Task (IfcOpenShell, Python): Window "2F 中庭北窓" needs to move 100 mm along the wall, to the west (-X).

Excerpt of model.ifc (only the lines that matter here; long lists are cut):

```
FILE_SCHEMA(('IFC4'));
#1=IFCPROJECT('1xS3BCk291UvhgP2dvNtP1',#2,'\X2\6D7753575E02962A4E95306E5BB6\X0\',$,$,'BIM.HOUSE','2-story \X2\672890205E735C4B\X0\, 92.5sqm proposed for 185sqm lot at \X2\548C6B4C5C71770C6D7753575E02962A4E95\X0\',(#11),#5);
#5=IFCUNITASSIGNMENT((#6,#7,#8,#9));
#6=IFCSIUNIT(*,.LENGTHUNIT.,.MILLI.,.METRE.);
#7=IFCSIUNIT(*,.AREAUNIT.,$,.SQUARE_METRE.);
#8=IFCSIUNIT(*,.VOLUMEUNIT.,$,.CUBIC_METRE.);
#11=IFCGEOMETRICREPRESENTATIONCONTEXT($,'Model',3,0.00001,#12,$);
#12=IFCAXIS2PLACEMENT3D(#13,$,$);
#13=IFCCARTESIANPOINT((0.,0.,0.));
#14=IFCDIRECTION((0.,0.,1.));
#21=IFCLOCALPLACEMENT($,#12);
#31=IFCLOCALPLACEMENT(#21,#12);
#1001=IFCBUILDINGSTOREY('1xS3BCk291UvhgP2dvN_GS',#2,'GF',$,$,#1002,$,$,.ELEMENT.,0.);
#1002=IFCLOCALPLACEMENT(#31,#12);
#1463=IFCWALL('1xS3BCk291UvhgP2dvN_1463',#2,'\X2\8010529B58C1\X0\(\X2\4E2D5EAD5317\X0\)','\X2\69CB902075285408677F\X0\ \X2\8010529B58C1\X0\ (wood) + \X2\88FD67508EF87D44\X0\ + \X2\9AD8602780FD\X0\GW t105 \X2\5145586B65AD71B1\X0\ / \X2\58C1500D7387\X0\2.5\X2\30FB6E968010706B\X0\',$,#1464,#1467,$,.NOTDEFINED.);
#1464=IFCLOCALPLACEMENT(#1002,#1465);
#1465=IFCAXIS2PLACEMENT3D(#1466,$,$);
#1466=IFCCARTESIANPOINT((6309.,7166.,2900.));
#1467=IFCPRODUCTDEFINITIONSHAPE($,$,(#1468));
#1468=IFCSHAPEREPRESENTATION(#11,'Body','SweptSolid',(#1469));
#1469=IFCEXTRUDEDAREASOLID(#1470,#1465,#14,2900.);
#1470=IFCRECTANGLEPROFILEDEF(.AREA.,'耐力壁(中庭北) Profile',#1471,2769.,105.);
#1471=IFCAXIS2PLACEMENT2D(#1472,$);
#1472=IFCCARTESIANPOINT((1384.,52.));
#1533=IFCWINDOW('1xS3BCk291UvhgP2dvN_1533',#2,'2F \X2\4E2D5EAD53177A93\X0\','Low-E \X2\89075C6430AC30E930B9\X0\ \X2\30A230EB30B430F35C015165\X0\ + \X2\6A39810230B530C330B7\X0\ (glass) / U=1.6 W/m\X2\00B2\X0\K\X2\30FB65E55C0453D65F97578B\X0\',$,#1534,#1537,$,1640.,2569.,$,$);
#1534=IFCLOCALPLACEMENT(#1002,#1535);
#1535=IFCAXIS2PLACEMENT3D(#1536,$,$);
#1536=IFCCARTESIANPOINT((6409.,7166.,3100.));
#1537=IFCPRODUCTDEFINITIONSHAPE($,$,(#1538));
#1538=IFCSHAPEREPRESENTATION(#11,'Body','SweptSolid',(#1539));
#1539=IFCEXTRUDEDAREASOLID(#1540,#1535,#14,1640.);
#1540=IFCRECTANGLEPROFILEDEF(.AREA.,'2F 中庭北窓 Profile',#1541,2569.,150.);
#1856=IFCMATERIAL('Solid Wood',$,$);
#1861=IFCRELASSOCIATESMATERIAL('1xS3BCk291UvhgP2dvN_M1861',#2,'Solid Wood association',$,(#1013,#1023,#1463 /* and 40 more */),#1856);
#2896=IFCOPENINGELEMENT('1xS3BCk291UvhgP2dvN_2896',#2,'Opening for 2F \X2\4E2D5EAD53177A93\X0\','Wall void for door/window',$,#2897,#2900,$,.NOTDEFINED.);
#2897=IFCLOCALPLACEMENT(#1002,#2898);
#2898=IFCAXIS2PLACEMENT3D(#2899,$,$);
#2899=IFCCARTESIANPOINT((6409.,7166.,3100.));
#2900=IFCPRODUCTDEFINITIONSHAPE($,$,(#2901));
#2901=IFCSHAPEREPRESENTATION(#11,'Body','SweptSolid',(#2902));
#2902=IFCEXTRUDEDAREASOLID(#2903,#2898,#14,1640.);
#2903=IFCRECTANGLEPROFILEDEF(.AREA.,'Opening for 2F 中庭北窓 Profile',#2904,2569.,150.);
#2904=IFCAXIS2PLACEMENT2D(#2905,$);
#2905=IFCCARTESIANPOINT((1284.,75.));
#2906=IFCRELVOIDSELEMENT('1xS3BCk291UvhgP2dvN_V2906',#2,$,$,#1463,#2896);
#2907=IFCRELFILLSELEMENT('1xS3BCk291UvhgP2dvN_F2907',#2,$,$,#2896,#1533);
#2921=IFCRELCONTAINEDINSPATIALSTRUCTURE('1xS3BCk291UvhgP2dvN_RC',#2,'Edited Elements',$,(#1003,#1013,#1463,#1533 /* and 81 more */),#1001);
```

```python
import ifcopenshell
import ifcopenshell.api.geometry
import ifcopenshell.util.placement
import ifcopenshell.util.unit

model = ifcopenshell.open("model.ifc")
unit_scale = ifcopenshell.util.unit.calculate_unit_scale(model)

window = model.by_guid("1xS3BCk291UvhgP2dvN_1533")
opening = window.FillsVoids[0].RelatingOpeningElement
wall = opening.VoidsElements[0].RelatingBuildingElement

wall_matrix = ifcopenshell.util.placement.get_local_placement(wall.ObjectPlacement)
shift = wall_matrix[:3, 0] * -0.1 / unit_scale
before = ifcopenshell.util.placement.get_local_placement(window.ObjectPlacement)[:3, 3].copy()

# The window is not placed relative to its opening, so move both.
for product in (opening, window):
    matrix = ifcopenshell.util.placement.get_local_placement(product.ObjectPlacement)
    matrix[:3, 3] += shift
    ifcopenshell.api.geometry.edit_object_placement(model, product=product, matrix=matrix, is_si=False)

after = ifcopenshell.util.placement.get_local_placement(window.ObjectPlacement)[:3, 3]
print("window moved by", (after - before).round(3) + 0.0)

model.write("model_updated.ifc")
```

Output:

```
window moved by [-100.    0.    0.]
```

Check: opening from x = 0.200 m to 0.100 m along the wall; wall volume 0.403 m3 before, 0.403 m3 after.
